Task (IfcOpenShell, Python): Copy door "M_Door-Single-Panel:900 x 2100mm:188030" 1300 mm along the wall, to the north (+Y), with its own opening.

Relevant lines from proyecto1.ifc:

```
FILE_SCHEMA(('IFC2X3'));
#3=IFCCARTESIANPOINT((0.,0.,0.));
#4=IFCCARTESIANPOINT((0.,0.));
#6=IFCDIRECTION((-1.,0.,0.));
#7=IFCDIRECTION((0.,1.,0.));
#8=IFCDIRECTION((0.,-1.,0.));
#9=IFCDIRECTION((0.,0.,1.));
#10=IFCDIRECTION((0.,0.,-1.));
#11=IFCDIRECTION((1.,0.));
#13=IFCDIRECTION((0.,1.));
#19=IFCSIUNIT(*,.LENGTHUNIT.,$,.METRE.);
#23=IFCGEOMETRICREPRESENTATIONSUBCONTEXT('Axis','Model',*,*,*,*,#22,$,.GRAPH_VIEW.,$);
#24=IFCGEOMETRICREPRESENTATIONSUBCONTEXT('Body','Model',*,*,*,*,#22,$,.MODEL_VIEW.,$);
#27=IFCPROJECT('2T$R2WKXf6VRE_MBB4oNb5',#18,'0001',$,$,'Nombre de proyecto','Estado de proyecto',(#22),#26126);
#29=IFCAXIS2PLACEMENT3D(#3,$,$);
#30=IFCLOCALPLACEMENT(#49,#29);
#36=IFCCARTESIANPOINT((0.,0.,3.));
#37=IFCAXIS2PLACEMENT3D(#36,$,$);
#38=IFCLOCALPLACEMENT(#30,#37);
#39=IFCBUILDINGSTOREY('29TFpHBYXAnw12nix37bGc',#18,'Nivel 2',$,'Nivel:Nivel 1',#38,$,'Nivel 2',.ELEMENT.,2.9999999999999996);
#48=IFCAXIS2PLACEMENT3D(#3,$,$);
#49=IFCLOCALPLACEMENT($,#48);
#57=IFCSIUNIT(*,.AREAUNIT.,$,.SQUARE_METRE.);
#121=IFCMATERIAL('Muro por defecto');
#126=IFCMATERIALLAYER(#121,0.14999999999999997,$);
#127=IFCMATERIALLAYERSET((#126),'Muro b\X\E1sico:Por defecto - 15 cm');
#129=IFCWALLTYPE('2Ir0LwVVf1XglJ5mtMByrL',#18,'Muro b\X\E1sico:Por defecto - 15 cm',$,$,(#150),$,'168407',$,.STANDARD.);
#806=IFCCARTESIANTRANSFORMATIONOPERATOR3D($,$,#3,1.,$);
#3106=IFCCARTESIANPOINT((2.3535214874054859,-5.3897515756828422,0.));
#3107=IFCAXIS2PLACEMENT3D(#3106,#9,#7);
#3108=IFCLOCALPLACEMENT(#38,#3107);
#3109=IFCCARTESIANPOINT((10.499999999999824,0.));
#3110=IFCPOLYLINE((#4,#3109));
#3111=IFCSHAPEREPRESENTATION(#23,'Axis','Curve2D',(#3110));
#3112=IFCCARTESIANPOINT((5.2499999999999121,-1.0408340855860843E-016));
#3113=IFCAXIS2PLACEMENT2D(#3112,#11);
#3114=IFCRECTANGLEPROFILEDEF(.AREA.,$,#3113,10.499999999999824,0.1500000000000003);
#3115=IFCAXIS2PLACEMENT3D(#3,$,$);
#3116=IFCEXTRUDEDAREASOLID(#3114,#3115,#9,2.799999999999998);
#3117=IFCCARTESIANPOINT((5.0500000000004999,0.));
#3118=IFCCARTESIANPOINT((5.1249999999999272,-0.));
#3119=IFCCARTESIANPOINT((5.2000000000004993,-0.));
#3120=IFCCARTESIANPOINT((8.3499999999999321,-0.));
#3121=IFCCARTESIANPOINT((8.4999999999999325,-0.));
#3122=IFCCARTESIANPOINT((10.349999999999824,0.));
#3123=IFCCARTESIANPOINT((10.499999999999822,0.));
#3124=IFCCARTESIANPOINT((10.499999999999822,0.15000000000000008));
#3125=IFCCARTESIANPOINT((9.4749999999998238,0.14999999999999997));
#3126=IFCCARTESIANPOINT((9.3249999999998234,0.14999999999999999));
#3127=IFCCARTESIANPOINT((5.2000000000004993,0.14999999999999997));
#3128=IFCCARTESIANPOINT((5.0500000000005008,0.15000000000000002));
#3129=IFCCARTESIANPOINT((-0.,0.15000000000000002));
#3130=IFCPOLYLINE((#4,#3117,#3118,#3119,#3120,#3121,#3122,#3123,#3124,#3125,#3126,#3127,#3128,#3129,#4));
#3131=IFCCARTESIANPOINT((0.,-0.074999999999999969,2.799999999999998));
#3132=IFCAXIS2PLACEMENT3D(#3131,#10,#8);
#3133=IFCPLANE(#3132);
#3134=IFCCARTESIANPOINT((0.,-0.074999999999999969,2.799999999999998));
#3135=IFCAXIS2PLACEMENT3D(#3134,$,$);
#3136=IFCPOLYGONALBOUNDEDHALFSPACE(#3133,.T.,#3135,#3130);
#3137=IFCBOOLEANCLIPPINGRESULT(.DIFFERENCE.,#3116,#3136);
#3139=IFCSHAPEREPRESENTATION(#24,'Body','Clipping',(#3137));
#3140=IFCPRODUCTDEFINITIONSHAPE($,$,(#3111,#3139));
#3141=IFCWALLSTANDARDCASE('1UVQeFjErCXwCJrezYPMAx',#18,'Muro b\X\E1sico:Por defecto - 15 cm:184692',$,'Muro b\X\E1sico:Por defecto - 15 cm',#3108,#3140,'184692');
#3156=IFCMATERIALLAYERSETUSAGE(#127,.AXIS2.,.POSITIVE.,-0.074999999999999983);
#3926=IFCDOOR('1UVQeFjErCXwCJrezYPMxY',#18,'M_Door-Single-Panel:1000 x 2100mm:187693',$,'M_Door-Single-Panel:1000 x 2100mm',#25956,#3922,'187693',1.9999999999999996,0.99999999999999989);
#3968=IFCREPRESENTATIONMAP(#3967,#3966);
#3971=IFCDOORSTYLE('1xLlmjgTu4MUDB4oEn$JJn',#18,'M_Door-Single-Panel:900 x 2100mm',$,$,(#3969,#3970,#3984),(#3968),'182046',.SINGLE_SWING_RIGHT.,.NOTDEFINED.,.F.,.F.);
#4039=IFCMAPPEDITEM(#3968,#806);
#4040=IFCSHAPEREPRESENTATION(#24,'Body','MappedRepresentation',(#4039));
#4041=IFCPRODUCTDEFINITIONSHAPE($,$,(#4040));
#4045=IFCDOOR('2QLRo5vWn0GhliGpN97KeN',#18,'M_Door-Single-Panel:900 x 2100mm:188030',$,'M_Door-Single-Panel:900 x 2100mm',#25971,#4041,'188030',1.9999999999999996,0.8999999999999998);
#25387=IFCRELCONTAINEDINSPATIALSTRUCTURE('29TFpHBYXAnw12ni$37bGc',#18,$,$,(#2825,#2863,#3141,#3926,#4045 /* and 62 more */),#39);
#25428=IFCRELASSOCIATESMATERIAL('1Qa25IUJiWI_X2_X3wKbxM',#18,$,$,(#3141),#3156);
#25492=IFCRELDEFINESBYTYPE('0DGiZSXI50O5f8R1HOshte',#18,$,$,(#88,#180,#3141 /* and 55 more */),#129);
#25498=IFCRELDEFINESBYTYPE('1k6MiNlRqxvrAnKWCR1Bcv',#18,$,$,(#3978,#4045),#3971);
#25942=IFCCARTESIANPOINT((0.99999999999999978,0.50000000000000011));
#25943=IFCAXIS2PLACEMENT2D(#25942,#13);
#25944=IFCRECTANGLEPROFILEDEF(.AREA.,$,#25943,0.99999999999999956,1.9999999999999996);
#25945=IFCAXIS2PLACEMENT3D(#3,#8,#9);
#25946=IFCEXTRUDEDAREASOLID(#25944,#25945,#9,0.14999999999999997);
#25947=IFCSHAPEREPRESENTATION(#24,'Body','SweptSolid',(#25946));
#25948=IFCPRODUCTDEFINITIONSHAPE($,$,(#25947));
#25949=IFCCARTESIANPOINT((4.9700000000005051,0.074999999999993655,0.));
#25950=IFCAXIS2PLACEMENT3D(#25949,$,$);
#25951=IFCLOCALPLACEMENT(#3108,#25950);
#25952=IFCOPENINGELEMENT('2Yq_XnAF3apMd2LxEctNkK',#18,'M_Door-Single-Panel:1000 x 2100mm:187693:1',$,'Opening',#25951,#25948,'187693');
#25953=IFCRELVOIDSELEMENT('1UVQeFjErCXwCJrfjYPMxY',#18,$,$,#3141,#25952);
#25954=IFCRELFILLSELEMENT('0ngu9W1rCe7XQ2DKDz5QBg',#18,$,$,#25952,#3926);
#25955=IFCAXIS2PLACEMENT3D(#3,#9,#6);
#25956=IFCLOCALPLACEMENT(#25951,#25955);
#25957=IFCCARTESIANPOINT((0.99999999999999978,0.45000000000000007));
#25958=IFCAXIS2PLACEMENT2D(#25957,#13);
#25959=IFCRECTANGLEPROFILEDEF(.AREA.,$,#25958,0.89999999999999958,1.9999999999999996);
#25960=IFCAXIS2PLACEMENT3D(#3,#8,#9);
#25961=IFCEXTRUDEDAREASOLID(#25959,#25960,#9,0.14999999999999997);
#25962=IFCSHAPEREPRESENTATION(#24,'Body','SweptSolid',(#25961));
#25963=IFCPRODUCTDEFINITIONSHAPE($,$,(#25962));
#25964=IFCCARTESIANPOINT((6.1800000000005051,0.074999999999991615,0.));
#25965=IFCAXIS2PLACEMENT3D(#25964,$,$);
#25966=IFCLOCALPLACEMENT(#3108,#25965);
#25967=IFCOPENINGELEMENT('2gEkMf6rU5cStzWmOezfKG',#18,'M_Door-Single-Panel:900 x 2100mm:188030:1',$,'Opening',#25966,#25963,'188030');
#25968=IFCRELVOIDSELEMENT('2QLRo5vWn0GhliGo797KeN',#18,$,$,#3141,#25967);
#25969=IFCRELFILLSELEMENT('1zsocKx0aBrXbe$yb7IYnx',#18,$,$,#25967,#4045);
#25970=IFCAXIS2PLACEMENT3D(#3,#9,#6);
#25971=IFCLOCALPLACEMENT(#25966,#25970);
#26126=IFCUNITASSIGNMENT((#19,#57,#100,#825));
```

```python
import ifcopenshell
import ifcopenshell.api.feature
import ifcopenshell.api.geometry
import ifcopenshell.api.root
import ifcopenshell.geom
import ifcopenshell.util.element
import ifcopenshell.util.placement
import ifcopenshell.util.shape
import ifcopenshell.util.unit

model = ifcopenshell.open("proyecto1.ifc")
unit_scale = ifcopenshell.util.unit.calculate_unit_scale(model)
settings = ifcopenshell.geom.settings()


def volume(element):
    """Net volume in cubic metres, openings subtracted."""
    shape = ifcopenshell.geom.create_shape(settings, element)
    return ifcopenshell.util.shape.get_volume(shape.geometry)


def reuse_history(source, copy):
    """copy_class also copies each property set's owner history, people and application; keep the originals."""
    for rel in copy.IsDefinedBy:
        if rel.is_a("IfcRelDefinesByProperties") and (history := rel.RelatingPropertyDefinition.OwnerHistory):
            rel.RelatingPropertyDefinition.OwnerHistory = source.OwnerHistory
            ifcopenshell.util.element.remove_deep2(model, history)


door = model.by_guid("2QLRo5vWn0GhliGpN97KeN")
opening = door.FillsVoids[0].RelatingOpeningElement
wall = opening.VoidsElements[0].RelatingBuildingElement
before = volume(wall)
shift = ifcopenshell.util.placement.get_local_placement(wall.ObjectPlacement)[:3, 0] * 1.3 / unit_scale

# copy_class copies the void relationship, type, container and properties, but no geometry.
new_opening = ifcopenshell.api.root.copy_class(model, product=opening)
new_opening.Representation = ifcopenshell.util.element.copy_deep(
    model, opening.Representation, exclude=["IfcGeometricRepresentationContext", "IfcRepresentationMap"]
)
new_opening.Name = "M_Door-Single-Panel:900 x 2100mm"
new_opening.Tag = None
new_door = ifcopenshell.api.root.copy_class(model, product=door)
new_door.Representation = ifcopenshell.util.element.copy_deep(
    model, door.Representation, exclude=["IfcGeometricRepresentationContext", "IfcRepresentationMap"]
)
new_door.Name = "M_Door-Single-Panel:900 x 2100mm"
new_door.Tag = None
reuse_history(door, new_door)
fills = ifcopenshell.api.feature.add_filling(model, opening=new_opening, element=new_door)
fills.OwnerHistory = new_door.OwnerHistory  # required in IFC2X3

for old, new in ((opening, new_opening), (door, new_door)):
    matrix = ifcopenshell.util.placement.get_local_placement(old.ObjectPlacement)
    matrix[:3, 3] += shift
    ifcopenshell.api.geometry.edit_object_placement(model, product=new, matrix=matrix, is_si=False)

after = volume(wall)

print(f"wall volume {before:.3f} -> {after:.3f} m3")

model.write("proyecto1_v2.ifc")
```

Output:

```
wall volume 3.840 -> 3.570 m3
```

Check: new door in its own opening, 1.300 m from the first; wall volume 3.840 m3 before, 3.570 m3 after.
